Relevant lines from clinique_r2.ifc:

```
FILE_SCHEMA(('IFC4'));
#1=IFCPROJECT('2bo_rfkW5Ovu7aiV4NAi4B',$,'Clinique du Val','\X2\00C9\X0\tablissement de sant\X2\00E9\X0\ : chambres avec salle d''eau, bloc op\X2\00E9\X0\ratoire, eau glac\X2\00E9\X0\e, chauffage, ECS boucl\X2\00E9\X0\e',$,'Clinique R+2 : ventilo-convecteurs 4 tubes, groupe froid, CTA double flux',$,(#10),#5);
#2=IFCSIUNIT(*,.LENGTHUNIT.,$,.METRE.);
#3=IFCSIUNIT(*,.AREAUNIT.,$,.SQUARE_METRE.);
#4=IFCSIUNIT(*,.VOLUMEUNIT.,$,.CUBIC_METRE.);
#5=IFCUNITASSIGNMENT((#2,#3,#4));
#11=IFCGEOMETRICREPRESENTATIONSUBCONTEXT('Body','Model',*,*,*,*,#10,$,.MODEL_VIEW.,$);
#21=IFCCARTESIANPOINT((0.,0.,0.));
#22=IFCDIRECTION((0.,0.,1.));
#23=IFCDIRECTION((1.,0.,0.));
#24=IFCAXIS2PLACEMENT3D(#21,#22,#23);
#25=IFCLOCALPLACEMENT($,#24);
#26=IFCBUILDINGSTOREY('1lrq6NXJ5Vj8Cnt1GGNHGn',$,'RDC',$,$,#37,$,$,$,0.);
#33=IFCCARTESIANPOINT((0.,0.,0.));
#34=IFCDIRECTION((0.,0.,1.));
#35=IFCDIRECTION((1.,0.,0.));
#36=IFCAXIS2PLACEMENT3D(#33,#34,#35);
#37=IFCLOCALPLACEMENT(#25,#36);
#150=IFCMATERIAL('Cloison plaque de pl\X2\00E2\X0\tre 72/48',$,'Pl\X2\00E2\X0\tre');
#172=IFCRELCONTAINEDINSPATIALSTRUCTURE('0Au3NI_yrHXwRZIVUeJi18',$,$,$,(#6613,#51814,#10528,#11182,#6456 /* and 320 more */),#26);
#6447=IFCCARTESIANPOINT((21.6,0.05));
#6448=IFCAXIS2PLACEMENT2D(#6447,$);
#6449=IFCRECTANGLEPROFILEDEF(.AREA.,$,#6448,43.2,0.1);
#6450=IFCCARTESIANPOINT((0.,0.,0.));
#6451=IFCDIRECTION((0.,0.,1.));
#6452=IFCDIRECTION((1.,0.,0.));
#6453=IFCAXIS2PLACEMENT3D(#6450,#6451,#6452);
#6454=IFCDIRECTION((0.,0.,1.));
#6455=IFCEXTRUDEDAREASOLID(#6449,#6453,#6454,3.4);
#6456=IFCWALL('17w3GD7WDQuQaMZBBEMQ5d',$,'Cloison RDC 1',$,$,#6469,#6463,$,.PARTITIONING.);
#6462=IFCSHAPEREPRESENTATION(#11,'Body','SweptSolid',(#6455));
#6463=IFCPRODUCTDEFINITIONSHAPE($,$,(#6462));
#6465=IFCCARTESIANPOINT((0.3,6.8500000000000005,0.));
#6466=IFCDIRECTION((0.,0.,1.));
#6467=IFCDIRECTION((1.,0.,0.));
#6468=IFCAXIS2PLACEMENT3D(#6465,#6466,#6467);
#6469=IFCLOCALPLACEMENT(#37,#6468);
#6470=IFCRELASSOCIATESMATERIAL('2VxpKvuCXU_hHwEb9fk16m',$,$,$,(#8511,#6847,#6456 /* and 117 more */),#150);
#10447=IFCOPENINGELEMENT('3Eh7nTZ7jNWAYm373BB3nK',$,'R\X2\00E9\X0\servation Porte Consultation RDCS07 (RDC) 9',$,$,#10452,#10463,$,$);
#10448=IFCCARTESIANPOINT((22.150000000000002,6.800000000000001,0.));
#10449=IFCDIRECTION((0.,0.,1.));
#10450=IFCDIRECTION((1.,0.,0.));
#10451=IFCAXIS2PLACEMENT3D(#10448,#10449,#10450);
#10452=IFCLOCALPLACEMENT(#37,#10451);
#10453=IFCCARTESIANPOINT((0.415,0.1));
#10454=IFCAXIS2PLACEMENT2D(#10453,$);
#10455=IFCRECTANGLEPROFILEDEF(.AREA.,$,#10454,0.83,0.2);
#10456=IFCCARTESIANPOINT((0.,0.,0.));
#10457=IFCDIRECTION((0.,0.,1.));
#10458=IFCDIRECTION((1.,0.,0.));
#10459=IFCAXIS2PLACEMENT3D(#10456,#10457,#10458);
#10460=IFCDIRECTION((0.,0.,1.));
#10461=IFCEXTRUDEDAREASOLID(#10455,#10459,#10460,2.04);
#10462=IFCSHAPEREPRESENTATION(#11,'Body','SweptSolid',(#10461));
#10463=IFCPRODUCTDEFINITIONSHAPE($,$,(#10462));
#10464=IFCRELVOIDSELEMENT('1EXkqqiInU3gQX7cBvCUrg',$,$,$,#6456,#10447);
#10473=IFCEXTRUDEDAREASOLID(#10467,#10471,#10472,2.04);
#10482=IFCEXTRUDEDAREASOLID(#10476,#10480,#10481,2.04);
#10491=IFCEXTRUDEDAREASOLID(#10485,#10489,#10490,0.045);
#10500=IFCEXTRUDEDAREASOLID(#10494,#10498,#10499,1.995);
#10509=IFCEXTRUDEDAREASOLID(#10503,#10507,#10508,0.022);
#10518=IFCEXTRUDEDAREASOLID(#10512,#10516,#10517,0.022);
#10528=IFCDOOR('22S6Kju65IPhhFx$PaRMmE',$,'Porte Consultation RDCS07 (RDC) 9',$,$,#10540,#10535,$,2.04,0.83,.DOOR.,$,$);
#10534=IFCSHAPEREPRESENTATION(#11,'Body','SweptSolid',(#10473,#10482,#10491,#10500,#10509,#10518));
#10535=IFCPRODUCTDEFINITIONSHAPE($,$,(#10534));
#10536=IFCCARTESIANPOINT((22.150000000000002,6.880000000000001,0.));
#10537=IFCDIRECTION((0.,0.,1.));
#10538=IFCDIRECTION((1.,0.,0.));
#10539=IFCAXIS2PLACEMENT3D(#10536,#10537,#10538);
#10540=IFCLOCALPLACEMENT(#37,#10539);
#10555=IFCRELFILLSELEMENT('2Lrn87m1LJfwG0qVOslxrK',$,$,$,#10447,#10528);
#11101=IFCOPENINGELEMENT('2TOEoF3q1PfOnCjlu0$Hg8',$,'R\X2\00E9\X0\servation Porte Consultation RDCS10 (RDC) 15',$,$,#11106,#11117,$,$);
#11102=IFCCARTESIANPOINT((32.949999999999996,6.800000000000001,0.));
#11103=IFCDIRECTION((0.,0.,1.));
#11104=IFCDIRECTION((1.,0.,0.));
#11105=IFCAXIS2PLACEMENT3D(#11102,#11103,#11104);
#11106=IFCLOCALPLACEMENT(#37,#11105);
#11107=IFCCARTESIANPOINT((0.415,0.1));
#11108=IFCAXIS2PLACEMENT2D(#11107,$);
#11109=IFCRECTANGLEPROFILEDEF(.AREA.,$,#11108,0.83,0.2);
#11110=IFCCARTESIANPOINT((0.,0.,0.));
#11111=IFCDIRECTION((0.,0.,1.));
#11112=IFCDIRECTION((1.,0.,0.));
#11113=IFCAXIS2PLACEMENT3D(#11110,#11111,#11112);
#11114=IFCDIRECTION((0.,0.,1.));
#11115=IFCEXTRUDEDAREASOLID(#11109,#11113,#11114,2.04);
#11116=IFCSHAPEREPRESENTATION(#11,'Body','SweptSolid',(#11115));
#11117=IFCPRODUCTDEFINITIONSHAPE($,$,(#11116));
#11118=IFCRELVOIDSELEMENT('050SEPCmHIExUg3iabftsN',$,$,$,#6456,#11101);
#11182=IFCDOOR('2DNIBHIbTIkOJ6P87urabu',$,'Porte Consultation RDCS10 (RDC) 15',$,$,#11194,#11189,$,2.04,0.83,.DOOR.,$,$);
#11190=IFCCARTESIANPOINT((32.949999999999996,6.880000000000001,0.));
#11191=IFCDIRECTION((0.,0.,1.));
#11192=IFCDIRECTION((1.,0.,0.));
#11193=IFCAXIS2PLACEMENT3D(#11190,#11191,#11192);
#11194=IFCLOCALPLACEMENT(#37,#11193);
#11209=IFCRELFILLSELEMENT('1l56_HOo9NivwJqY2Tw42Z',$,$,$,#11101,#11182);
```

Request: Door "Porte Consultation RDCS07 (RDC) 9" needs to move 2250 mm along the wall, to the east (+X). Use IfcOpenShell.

```python
import ifcopenshell
import ifcopenshell.api.geometry
import ifcopenshell.util.placement
import ifcopenshell.util.unit

model = ifcopenshell.open("clinique_r2.ifc")
unit_scale = ifcopenshell.util.unit.calculate_unit_scale(model)

door = model.by_id(10528)
opening = door.FillsVoids[0].RelatingOpeningElement
wall = opening.VoidsElements[0].RelatingBuildingElement

wall_matrix = ifcopenshell.util.placement.get_local_placement(wall.ObjectPlacement)
shift = wall_matrix[:3, 0] * 2.25 / unit_scale
before = ifcopenshell.util.placement.get_local_placement(door.ObjectPlacement)[:3, 3].copy()

# The door is not placed relative to its opening, so move both.
for product in (opening, door):
    matrix = ifcopenshell.util.placement.get_local_placement(product.ObjectPlacement)
    matrix[:3, 3] += shift
    ifcopenshell.api.geometry.edit_object_placement(model, product=product, matrix=matrix, is_si=False)

after = ifcopenshell.util.placement.get_local_placement(door.ObjectPlacement)[:3, 3]
print("door moved by", (after - before).round(3) + 0.0)

model.write("clinique_r2_updated.ifc")
```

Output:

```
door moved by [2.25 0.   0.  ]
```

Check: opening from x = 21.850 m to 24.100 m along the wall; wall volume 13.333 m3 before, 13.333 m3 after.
